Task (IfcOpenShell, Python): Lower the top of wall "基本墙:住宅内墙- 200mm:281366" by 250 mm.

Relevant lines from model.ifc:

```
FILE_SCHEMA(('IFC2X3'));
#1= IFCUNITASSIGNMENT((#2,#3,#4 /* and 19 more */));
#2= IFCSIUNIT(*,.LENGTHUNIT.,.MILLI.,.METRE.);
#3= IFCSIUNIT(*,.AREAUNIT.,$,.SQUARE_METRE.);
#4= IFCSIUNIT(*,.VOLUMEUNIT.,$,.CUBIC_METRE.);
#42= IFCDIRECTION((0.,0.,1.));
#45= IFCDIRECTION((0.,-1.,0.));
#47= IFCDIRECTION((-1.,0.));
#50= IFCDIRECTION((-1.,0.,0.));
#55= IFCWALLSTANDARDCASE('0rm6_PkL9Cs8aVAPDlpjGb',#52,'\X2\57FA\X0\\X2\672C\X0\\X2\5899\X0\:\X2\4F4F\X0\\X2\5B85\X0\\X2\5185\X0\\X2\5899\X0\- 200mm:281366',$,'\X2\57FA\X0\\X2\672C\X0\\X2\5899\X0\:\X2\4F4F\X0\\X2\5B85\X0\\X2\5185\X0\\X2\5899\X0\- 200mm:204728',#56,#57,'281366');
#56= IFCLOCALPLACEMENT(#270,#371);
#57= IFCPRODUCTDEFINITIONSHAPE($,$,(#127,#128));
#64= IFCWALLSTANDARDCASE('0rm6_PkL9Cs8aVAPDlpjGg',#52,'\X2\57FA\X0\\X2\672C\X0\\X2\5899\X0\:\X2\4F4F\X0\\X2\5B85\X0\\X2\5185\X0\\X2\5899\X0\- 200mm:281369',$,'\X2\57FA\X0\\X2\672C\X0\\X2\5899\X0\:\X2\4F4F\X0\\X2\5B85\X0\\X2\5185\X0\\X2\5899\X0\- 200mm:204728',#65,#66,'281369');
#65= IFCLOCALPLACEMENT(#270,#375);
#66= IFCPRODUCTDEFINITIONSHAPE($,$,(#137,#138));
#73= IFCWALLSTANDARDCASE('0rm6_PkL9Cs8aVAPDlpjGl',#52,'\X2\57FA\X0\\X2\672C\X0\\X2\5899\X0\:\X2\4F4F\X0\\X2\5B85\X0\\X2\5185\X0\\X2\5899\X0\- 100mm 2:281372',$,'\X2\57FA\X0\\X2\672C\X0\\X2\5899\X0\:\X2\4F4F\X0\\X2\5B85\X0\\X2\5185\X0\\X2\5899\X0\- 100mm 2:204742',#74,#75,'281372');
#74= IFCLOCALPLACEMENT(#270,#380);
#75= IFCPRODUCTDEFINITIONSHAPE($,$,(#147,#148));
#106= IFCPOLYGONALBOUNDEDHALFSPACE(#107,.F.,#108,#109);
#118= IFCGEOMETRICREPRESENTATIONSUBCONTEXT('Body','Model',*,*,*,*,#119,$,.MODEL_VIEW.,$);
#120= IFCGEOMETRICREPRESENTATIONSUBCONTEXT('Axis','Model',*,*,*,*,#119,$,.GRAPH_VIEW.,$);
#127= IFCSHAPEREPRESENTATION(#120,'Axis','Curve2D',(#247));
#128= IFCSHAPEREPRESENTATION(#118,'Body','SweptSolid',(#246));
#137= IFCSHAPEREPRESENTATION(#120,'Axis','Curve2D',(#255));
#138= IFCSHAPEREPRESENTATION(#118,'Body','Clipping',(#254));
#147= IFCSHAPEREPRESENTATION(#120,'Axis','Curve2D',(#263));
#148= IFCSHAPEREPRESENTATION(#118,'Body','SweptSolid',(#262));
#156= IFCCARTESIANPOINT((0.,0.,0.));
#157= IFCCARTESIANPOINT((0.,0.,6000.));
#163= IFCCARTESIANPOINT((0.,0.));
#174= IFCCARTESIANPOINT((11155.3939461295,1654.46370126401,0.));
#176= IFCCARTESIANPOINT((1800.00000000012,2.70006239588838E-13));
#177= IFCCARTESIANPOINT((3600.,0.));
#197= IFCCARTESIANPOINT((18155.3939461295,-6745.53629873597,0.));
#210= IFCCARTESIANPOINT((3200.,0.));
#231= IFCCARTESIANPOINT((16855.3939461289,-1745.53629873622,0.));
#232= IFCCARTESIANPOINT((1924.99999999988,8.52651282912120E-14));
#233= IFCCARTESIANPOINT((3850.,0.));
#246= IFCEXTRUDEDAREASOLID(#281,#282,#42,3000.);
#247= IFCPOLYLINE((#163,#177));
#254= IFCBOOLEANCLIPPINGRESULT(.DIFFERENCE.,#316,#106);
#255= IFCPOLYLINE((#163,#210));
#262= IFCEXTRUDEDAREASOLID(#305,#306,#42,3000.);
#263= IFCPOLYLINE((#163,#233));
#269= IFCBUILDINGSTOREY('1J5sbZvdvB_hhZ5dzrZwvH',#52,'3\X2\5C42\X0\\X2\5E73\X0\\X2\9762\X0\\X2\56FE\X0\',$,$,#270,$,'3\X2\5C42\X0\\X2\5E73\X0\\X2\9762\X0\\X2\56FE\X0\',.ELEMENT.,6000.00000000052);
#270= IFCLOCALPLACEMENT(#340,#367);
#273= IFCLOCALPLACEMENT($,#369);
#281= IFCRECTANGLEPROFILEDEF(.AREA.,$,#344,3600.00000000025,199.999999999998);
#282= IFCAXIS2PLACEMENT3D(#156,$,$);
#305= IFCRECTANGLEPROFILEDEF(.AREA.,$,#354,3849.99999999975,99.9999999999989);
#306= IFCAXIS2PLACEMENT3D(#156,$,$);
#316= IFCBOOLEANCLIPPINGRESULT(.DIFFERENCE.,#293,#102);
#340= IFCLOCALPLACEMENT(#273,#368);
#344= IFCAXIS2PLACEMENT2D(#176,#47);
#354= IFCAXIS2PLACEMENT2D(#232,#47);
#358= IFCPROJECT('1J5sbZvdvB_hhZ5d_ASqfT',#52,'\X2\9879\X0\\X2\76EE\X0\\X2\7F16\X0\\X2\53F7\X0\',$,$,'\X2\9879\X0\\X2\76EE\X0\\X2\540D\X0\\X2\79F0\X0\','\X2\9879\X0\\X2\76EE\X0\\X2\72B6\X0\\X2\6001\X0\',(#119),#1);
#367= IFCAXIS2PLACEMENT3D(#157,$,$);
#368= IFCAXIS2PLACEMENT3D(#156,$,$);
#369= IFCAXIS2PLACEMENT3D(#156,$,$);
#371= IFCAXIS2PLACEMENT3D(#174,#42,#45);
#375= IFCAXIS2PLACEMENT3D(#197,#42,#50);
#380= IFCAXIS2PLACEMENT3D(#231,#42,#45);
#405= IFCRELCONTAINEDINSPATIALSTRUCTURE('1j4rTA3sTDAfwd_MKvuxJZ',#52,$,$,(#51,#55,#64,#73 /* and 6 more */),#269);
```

```python
import ifcopenshell
import ifcopenshell.geom
import ifcopenshell.util.representation
import ifcopenshell.util.shape

model = ifcopenshell.open("model.ifc")
settings = ifcopenshell.geom.settings()


def volume(element):
    """Net volume in cubic metres, openings subtracted."""
    shape = ifcopenshell.geom.create_shape(settings, element)
    return ifcopenshell.util.shape.get_volume(shape.geometry)


wall = model.by_guid("0rm6_PkL9Cs8aVAPDlpjGb")
before = volume(wall)

body = ifcopenshell.util.representation.get_representation(wall, "Model", "Body")
solid = body.Items[0]
old_height = solid.Depth
solid.Depth -= 250.0
after = volume(wall)

print(f"height {old_height:g} -> {solid.Depth:g}, volume {before:.3f} -> {after:.3f} m3")

model.write("model_rev.ifc")
```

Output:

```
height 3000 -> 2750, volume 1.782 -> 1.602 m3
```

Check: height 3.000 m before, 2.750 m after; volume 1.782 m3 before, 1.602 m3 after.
